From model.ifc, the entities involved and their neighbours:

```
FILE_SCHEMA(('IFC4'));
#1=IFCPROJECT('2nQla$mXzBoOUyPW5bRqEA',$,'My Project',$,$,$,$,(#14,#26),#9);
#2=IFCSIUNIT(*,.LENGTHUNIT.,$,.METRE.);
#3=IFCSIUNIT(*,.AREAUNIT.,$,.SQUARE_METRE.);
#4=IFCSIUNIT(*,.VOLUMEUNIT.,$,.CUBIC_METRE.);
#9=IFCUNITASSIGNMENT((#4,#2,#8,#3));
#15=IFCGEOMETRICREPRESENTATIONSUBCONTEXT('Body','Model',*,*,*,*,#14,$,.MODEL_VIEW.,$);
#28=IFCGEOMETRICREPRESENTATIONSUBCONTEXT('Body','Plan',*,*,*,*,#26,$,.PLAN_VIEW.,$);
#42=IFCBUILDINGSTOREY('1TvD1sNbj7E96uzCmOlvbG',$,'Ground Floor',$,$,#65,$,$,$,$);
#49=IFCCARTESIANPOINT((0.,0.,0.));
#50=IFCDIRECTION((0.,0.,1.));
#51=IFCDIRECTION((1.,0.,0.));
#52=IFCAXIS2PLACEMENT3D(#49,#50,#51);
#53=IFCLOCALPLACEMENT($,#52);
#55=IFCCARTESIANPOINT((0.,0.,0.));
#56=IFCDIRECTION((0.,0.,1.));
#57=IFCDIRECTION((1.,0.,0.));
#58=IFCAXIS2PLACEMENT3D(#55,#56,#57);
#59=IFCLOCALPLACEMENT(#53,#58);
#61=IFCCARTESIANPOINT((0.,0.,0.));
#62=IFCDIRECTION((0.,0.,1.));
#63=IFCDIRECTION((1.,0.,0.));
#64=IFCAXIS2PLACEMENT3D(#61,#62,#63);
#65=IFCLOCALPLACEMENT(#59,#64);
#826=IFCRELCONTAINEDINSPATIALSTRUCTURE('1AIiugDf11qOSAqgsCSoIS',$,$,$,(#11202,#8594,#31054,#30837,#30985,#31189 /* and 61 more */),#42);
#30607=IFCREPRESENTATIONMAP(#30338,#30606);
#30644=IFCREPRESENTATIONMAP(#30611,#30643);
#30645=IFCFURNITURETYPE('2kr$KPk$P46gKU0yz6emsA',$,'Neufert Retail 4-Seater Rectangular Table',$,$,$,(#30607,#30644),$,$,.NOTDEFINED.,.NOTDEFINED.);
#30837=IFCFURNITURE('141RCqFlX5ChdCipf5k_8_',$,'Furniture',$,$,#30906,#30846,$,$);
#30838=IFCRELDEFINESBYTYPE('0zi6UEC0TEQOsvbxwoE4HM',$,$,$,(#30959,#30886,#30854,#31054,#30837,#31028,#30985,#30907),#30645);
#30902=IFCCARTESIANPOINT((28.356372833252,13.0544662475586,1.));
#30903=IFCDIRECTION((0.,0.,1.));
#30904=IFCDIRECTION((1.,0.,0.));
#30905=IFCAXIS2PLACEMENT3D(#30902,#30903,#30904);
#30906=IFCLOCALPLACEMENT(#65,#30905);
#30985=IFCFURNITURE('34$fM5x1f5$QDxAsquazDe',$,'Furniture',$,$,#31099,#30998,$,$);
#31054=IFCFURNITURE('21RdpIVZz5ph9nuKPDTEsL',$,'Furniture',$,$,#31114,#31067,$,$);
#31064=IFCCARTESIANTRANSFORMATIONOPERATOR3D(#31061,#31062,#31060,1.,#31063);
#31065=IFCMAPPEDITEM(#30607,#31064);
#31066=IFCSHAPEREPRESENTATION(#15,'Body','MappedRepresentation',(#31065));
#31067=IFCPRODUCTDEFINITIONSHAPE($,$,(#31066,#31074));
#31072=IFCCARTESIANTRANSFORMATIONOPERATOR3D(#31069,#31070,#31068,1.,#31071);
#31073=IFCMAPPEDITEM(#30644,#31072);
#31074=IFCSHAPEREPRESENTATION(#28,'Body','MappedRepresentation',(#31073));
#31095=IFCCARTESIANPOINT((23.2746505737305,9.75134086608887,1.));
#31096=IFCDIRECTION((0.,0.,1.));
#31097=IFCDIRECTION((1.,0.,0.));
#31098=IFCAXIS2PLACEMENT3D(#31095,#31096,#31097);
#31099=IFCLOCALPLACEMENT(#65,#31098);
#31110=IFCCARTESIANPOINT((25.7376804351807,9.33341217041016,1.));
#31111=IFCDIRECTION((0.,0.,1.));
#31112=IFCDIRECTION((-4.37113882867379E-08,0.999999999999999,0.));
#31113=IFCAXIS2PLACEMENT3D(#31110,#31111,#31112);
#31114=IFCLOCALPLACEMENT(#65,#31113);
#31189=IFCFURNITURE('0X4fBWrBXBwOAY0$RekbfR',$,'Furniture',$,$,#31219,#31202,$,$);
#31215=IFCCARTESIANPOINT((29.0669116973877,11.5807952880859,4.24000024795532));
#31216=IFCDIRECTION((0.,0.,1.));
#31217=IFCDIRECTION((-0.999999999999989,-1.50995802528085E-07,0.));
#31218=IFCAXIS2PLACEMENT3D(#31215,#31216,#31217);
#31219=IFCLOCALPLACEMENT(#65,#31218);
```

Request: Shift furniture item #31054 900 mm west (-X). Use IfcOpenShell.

```python
import ifcopenshell
import ifcopenshell.api.geometry
import ifcopenshell.util.placement

model = ifcopenshell.open("model.ifc")

item = model.by_guid("21RdpIVZz5ph9nuKPDTEsL")
matrix = ifcopenshell.util.placement.get_local_placement(item.ObjectPlacement)
matrix[0, 3] -= 0.9
ifcopenshell.api.geometry.edit_object_placement(model, product=item, matrix=matrix, is_si=False)

print(ifcopenshell.util.placement.get_local_placement(item.ObjectPlacement).round(3) + 0.0)

model.write("model_rev.ifc")
```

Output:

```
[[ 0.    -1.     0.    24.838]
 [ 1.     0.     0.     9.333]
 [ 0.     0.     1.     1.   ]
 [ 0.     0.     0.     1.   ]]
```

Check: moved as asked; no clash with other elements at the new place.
